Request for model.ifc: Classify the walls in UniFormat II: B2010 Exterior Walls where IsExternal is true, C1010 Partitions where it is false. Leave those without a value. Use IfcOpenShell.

First a look at what the model holds.

```python
import ifcopenshell
import ifcopenshell.util.element

model = ifcopenshell.open("model.ifc")
print(model.schema)
print("classifications:", [c.Name for c in model.by_type("IfcClassification")])
values = [ifcopenshell.util.element.get_pset(e, "Pset_WallCommon", "IsExternal") for e in model.by_type("IfcWall")]
for value in (True, False, None):
    print("IsExternal", value, values.count(value))
```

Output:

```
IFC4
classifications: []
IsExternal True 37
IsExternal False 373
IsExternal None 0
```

```python
import ifcopenshell
import ifcopenshell.api.classification
import ifcopenshell.util.element

model = ifcopenshell.open("model.ifc")

system = ifcopenshell.api.classification.add_classification(model, classification="UniFormat II")

walls = model.by_type("IfcWall")
external = {e: ifcopenshell.util.element.get_pset(e, "Pset_WallCommon", "IsExternal") for e in walls}
for flag, code, name in ((True, "B2010", "Exterior Walls"), (False, "C1010", "Partitions")):
    products = [e for e in walls if external[e] is flag]
    ifcopenshell.api.classification.add_reference(
        model, products=products, classification=system, identification=code, name=name
    )
    print(code, len(products))

model.write("model_rev.ifc")
```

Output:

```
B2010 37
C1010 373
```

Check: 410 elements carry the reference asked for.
